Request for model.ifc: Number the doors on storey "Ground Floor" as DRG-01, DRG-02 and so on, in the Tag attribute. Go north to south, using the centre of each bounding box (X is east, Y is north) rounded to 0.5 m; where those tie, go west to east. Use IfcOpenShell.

First a look at what the model holds.

```python
import ifcopenshell
import ifcopenshell.util.element
import ifcopenshell.util.placement

model = ifcopenshell.open("model.ifc")
print(model.schema)
storey = next(s for s in model.by_type("IfcBuildingStorey") if s.Name == "Ground Floor")
doors = [e for e in ifcopenshell.util.element.get_decomposition(storey) if e.is_a("IfcDoor")]
for e in sorted(doors, key=lambda e: e.id()):
    origin = ifcopenshell.util.placement.get_local_placement(e.ObjectPlacement)[:3, 3]
    print(e.id(), e.Tag, e.Name, origin.round(2) + 0.0, sep=" | ")
```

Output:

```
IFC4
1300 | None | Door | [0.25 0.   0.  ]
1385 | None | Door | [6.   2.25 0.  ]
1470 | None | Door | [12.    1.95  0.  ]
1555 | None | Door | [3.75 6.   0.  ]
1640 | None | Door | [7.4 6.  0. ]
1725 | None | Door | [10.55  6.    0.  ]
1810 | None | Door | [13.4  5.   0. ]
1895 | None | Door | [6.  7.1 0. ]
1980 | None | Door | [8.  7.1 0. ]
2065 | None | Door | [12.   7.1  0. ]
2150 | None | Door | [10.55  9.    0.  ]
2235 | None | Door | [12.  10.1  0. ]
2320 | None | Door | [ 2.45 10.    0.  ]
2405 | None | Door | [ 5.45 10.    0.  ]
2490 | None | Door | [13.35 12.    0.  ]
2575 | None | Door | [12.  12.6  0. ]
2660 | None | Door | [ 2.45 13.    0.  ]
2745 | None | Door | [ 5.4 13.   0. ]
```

```python
import ifcopenshell
import ifcopenshell.geom
import ifcopenshell.util.element
import ifcopenshell.util.shape

model = ifcopenshell.open("model.ifc")
settings = ifcopenshell.geom.settings()
settings.set("use-world-coords", True)


def centre(element):
    shape = ifcopenshell.geom.create_shape(settings, element)
    return ifcopenshell.util.shape.get_bbox_centroid(shape.geometry)


storey = next(s for s in model.by_type("IfcBuildingStorey") if s.Name == "Ground Floor")
doors = [e for e in ifcopenshell.util.element.get_decomposition(storey) if e.is_a("IfcDoor")]

# Insertion points can sit at a corner or the storey origin, so sort by the geometry (in metres).
centres = {e: centre(e) for e in doors}
doors.sort(key=lambda e: (-round(centres[e][1] / 0.5), centres[e][0]))

for i, e in enumerate(doors, start=1):
    number = f"DRG-{i:02d}"
    e.Tag = number
    print(e.id(), number)

model.write("model-out.ifc")
```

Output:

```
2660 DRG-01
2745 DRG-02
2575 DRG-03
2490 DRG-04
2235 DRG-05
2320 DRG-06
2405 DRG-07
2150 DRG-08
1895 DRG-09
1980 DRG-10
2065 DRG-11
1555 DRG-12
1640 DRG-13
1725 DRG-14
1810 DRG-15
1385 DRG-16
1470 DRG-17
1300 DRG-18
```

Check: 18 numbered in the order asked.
